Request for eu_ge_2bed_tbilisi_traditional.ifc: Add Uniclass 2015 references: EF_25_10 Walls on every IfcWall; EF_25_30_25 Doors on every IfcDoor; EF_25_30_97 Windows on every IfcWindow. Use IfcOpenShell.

First a look at what the model holds.

```python
import ifcopenshell

model = ifcopenshell.open("eu_ge_2bed_tbilisi_traditional.ifc")
print(model.schema)
print("classifications:", [c.Name for c in model.by_type("IfcClassification")])
for ifc_class in ("IfcDoor", "IfcRoof", "IfcStair", "IfcWall", "IfcWindow"):
    print(ifc_class, len(model.by_type(ifc_class)))
```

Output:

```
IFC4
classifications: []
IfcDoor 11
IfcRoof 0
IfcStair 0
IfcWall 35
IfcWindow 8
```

```python
import ifcopenshell
import ifcopenshell.api.classification

model = ifcopenshell.open("eu_ge_2bed_tbilisi_traditional.ifc")

system = ifcopenshell.api.classification.add_classification(model, classification="Uniclass 2015")

codes = {
    "IfcWall": ("EF_25_10", "Walls"),
    "IfcDoor": ("EF_25_30_25", "Doors"),
    "IfcWindow": ("EF_25_30_97", "Windows"),
}
for ifc_class, (code, name) in codes.items():
    products = model.by_type(ifc_class)
    ifcopenshell.api.classification.add_reference(
        model, products=products, classification=system, identification=code, name=name
    )
    print(code, len(products))

model.write("eu_ge_2bed_tbilisi_traditional_rev.ifc")
```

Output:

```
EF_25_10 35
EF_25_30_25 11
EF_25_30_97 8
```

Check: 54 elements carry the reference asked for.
